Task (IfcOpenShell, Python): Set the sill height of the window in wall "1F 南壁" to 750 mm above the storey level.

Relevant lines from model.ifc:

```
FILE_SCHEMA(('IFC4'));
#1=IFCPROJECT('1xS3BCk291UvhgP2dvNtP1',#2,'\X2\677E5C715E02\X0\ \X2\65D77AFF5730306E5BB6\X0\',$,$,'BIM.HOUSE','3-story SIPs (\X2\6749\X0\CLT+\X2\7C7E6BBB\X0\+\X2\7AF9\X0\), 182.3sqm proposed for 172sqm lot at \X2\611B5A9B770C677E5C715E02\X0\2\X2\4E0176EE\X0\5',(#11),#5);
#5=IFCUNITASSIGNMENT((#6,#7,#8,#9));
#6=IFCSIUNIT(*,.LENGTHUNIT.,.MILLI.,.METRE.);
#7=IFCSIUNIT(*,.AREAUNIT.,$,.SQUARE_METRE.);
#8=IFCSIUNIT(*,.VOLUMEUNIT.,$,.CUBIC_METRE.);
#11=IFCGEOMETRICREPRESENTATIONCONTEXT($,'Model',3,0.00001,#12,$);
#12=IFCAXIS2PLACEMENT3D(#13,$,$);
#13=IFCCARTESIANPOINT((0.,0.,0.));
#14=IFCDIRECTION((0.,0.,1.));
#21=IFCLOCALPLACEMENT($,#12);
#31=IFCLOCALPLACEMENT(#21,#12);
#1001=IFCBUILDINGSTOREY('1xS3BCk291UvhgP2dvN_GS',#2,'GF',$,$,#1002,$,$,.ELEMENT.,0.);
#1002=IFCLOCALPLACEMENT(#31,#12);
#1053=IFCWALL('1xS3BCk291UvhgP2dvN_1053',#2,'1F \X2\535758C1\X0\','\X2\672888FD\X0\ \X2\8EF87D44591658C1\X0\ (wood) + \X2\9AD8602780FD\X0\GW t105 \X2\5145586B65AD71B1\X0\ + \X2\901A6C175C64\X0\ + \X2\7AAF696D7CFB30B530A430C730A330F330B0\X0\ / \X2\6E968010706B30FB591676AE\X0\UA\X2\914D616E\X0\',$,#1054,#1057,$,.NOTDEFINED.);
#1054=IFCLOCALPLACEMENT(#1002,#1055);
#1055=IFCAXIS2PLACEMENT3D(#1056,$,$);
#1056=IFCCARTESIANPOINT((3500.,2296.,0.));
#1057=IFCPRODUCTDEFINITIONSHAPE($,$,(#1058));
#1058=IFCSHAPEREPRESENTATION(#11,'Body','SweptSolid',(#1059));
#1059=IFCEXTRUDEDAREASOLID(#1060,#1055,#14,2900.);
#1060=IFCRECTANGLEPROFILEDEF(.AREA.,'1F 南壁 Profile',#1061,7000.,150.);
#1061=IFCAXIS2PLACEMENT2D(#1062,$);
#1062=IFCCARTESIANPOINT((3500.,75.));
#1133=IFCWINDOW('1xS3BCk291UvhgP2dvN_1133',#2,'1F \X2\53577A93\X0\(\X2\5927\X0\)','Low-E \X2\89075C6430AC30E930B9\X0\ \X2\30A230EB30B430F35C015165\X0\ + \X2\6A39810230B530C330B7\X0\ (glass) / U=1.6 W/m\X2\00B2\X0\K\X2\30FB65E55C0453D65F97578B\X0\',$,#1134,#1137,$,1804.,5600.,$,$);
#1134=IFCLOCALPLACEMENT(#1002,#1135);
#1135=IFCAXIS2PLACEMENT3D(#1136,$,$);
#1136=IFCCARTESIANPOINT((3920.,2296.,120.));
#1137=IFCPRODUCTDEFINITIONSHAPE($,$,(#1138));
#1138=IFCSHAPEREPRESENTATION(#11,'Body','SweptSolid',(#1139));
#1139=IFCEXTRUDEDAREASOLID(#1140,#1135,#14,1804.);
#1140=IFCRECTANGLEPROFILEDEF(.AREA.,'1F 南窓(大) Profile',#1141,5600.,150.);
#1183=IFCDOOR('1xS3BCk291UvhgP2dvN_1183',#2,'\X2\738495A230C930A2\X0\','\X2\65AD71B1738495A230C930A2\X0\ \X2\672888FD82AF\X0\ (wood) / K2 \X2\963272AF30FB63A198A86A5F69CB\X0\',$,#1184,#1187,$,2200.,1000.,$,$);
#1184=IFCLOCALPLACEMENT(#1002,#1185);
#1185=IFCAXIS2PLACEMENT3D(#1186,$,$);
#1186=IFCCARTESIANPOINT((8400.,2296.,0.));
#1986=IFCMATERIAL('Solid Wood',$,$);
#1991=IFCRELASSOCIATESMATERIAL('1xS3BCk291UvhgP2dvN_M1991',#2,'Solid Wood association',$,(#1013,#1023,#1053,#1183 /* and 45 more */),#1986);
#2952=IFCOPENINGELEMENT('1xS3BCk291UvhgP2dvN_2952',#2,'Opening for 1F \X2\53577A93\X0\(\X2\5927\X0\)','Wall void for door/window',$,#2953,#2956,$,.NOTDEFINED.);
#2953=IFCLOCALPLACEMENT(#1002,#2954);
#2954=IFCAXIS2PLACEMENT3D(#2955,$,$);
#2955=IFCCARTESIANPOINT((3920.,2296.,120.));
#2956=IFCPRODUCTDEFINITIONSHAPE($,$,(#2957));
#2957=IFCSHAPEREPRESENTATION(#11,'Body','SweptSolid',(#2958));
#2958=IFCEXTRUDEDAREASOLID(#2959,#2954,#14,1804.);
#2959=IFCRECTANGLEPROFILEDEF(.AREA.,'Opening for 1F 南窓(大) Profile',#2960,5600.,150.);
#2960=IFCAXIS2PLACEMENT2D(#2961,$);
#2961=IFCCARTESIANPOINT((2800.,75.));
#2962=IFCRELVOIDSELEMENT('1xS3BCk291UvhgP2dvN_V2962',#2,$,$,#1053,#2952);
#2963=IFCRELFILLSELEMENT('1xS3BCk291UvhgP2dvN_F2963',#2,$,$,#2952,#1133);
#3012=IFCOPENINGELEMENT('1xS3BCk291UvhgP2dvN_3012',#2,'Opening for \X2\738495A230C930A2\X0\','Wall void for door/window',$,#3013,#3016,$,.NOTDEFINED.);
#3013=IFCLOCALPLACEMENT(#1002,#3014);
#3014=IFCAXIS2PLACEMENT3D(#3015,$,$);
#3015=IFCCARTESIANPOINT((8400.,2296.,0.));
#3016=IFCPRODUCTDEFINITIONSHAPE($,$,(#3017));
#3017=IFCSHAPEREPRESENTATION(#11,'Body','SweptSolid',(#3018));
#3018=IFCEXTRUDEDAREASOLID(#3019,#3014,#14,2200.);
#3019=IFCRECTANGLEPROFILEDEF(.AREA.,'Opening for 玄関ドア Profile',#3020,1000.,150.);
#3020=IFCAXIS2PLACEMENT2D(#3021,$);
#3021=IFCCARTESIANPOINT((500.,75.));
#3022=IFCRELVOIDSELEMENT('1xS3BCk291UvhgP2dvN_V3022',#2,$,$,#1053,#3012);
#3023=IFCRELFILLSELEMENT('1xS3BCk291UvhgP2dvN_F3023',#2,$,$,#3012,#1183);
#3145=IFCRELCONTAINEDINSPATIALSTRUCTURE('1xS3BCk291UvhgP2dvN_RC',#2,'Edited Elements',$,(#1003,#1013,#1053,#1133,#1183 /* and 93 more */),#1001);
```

```python
import numpy as np
import ifcopenshell
import ifcopenshell.api.geometry
import ifcopenshell.geom
import ifcopenshell.util.element
import ifcopenshell.util.placement
import ifcopenshell.util.shape
import ifcopenshell.util.unit

model = ifcopenshell.open("model.ifc")
unit_scale = ifcopenshell.util.unit.calculate_unit_scale(model)

window = model.by_id(1133)
opening = window.FillsVoids[0].RelatingOpeningElement
storey = ifcopenshell.util.element.get_container(window, ifc_class="IfcBuildingStorey")
level = ifcopenshell.util.placement.get_local_placement(storey.ObjectPlacement)[2, 3]

# The opening's origin need not be at the sill, so measure its lowest point.
shape = ifcopenshell.geom.create_shape(ifcopenshell.geom.settings(), opening)
bottom = ifcopenshell.util.shape.get_shape_bottom_elevation(shape, shape.geometry) / unit_scale
dz = level + 750.0 - bottom

shift = np.array([0.0, 0.0, dz])
# The window is not placed relative to its opening, so move both.
for product in (opening, window):
    matrix = ifcopenshell.util.placement.get_local_placement(product.ObjectPlacement)
    matrix[:3, 3] += shift
    ifcopenshell.api.geometry.edit_object_placement(model, product=product, matrix=matrix, is_si=False)

print(f"moved by {dz * unit_scale:+.3f} m")

model.write("model_updated.ifc")
```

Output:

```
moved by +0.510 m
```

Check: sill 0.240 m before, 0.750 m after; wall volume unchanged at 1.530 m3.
